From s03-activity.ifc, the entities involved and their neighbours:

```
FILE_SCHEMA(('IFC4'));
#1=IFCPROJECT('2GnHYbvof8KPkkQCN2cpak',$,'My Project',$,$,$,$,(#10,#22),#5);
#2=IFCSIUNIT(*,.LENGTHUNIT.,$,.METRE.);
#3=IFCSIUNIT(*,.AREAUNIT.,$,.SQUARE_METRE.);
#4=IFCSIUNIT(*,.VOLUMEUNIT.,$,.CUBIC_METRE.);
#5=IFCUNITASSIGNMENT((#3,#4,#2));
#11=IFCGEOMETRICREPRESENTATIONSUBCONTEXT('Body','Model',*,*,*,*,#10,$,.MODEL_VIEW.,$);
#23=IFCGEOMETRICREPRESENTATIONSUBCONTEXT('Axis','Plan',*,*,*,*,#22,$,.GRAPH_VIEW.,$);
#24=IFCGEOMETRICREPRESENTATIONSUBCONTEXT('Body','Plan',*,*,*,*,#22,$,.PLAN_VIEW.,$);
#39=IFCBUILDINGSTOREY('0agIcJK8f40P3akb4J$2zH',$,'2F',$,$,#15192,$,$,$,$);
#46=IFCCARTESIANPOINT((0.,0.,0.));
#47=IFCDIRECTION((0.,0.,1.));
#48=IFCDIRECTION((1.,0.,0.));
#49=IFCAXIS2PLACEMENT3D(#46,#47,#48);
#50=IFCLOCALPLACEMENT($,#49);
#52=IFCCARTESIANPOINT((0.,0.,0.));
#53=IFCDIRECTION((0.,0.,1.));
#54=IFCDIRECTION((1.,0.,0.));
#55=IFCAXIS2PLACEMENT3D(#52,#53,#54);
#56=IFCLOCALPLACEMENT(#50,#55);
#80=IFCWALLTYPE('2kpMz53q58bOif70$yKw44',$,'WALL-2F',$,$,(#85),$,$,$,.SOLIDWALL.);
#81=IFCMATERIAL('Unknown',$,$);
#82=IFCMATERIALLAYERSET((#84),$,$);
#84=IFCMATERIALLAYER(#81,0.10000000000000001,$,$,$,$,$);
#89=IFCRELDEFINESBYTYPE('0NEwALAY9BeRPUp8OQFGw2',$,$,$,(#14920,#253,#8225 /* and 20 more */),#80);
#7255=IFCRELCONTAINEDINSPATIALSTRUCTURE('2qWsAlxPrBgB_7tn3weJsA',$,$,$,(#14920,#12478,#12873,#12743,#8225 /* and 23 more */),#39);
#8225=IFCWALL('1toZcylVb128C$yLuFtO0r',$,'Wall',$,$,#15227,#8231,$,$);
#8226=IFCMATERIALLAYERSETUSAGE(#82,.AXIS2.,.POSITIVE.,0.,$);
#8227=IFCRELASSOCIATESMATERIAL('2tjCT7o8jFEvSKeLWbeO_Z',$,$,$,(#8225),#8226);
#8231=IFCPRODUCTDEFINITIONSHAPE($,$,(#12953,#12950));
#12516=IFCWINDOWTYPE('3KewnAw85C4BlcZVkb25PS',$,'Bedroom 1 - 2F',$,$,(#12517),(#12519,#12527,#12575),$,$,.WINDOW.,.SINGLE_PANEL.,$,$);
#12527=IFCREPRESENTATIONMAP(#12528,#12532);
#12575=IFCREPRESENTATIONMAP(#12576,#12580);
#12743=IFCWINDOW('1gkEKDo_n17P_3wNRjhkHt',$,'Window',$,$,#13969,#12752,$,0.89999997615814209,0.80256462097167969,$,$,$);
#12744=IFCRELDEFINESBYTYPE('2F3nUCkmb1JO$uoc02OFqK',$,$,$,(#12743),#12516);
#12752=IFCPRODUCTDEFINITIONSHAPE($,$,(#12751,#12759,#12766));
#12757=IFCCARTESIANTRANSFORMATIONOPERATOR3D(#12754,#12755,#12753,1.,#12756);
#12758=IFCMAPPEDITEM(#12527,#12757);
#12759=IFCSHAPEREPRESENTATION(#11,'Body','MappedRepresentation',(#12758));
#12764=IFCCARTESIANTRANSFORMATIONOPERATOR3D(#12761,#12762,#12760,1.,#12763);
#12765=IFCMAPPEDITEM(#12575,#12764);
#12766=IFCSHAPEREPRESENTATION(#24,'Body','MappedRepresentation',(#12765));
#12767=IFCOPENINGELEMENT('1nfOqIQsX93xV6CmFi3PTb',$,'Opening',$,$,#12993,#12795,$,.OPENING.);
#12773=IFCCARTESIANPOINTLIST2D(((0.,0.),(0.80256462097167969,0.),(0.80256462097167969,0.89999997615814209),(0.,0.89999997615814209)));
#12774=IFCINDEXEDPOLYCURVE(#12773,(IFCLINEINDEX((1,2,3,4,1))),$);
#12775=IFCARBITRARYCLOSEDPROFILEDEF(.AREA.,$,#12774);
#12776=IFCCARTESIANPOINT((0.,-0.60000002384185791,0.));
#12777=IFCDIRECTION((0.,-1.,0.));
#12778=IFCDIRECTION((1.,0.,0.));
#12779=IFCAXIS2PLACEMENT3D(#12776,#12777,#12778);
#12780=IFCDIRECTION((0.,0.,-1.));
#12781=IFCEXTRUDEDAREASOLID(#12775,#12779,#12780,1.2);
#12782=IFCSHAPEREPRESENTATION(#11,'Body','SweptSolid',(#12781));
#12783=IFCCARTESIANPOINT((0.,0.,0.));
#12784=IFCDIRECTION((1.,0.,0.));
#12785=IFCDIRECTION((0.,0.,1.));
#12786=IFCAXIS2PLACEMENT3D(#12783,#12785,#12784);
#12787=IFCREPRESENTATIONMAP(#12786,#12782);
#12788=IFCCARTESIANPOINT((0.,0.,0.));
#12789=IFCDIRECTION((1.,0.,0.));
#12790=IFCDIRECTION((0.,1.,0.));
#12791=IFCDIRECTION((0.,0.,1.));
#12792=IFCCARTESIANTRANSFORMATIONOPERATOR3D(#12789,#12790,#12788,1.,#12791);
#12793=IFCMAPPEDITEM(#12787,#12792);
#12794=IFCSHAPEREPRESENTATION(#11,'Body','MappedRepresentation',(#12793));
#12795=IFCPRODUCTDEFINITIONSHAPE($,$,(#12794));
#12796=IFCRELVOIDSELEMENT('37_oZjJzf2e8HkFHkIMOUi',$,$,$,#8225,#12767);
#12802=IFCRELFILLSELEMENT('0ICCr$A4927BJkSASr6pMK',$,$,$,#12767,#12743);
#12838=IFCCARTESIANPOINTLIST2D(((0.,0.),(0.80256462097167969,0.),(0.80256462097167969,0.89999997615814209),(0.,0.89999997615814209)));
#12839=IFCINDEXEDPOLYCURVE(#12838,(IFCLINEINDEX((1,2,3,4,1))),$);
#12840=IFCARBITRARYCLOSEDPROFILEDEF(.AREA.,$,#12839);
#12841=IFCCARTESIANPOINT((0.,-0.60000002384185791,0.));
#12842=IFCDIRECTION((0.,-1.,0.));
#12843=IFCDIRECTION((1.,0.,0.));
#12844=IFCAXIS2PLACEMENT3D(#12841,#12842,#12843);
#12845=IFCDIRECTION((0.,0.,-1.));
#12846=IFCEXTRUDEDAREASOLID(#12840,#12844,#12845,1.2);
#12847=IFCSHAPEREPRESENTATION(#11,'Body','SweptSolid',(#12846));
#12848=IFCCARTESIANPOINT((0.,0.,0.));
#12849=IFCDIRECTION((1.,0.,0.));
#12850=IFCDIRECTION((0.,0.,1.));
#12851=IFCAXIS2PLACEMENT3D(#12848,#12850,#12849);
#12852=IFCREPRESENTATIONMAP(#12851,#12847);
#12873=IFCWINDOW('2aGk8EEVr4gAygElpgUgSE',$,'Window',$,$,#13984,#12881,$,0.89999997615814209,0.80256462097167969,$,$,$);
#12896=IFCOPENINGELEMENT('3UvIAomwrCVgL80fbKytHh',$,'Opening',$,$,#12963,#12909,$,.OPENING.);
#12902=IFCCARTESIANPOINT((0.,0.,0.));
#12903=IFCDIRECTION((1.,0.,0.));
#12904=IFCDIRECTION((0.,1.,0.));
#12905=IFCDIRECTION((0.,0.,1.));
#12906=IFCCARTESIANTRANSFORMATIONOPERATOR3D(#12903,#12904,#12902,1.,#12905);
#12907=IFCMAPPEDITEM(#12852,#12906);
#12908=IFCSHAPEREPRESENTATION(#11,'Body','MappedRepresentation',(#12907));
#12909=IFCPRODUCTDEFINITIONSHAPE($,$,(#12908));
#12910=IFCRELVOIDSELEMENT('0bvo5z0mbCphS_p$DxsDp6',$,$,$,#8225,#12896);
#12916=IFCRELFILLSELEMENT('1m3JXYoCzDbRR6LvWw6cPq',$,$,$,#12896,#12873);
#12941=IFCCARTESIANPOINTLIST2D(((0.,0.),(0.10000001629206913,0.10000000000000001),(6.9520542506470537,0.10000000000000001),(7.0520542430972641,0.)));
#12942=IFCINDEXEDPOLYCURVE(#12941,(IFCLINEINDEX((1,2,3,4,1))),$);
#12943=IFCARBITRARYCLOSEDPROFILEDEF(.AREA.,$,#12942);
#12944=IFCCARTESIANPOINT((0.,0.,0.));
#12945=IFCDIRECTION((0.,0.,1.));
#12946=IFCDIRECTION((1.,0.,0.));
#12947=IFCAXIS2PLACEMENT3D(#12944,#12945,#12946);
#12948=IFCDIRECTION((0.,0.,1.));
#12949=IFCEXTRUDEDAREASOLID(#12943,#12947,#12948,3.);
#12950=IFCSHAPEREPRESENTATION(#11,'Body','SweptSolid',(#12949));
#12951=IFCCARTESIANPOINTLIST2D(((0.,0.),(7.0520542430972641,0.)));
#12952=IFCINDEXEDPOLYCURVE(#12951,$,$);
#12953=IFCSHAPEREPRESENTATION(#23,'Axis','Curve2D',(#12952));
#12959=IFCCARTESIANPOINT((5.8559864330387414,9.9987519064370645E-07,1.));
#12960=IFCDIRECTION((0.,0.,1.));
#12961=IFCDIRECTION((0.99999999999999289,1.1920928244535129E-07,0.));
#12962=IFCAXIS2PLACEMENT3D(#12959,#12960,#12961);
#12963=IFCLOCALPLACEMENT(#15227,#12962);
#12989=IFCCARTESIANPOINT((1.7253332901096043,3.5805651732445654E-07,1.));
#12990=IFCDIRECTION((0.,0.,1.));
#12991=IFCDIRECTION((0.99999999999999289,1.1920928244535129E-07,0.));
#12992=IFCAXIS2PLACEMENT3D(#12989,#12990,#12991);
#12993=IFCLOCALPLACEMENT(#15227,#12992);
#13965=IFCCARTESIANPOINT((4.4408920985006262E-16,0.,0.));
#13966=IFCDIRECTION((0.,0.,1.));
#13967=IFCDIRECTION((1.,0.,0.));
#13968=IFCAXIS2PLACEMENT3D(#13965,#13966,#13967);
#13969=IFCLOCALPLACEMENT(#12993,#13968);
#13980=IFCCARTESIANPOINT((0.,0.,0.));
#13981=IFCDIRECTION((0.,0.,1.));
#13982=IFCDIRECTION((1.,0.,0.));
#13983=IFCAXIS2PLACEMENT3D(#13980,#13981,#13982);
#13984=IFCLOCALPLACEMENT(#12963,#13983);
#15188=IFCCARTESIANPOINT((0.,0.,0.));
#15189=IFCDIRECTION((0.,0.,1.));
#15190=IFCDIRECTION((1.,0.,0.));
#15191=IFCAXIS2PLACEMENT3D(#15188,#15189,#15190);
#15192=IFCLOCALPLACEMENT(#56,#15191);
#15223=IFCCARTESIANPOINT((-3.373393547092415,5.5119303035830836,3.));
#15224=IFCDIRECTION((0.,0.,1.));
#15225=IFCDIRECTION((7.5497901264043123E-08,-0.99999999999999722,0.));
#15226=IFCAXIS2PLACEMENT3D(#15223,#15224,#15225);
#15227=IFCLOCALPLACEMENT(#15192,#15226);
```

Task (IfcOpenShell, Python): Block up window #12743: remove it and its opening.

```python
import ifcopenshell
import ifcopenshell.api.feature
import ifcopenshell.api.root
import ifcopenshell.geom
import ifcopenshell.util.shape

model = ifcopenshell.open("s03-activity.ifc")
settings = ifcopenshell.geom.settings()


def volume(element):
    """Net volume in cubic metres, openings subtracted."""
    shape = ifcopenshell.geom.create_shape(settings, element)
    return ifcopenshell.util.shape.get_volume(shape.geometry)


window = model.by_guid("1gkEKDo_n17P_3wNRjhkHt")
opening = window.FillsVoids[0].RelatingOpeningElement
wall = opening.VoidsElements[0].RelatingBuildingElement
before = volume(wall)

ifcopenshell.api.root.remove_product(model, product=window)
ifcopenshell.api.feature.remove_feature(model, feature=opening)

after = volume(wall)

print(f"wall volume {before:.3f} -> {after:.3f} m3")

model.write("s03-activity_rev.ifc")
```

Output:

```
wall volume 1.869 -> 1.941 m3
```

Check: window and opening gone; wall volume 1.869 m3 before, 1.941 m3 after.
